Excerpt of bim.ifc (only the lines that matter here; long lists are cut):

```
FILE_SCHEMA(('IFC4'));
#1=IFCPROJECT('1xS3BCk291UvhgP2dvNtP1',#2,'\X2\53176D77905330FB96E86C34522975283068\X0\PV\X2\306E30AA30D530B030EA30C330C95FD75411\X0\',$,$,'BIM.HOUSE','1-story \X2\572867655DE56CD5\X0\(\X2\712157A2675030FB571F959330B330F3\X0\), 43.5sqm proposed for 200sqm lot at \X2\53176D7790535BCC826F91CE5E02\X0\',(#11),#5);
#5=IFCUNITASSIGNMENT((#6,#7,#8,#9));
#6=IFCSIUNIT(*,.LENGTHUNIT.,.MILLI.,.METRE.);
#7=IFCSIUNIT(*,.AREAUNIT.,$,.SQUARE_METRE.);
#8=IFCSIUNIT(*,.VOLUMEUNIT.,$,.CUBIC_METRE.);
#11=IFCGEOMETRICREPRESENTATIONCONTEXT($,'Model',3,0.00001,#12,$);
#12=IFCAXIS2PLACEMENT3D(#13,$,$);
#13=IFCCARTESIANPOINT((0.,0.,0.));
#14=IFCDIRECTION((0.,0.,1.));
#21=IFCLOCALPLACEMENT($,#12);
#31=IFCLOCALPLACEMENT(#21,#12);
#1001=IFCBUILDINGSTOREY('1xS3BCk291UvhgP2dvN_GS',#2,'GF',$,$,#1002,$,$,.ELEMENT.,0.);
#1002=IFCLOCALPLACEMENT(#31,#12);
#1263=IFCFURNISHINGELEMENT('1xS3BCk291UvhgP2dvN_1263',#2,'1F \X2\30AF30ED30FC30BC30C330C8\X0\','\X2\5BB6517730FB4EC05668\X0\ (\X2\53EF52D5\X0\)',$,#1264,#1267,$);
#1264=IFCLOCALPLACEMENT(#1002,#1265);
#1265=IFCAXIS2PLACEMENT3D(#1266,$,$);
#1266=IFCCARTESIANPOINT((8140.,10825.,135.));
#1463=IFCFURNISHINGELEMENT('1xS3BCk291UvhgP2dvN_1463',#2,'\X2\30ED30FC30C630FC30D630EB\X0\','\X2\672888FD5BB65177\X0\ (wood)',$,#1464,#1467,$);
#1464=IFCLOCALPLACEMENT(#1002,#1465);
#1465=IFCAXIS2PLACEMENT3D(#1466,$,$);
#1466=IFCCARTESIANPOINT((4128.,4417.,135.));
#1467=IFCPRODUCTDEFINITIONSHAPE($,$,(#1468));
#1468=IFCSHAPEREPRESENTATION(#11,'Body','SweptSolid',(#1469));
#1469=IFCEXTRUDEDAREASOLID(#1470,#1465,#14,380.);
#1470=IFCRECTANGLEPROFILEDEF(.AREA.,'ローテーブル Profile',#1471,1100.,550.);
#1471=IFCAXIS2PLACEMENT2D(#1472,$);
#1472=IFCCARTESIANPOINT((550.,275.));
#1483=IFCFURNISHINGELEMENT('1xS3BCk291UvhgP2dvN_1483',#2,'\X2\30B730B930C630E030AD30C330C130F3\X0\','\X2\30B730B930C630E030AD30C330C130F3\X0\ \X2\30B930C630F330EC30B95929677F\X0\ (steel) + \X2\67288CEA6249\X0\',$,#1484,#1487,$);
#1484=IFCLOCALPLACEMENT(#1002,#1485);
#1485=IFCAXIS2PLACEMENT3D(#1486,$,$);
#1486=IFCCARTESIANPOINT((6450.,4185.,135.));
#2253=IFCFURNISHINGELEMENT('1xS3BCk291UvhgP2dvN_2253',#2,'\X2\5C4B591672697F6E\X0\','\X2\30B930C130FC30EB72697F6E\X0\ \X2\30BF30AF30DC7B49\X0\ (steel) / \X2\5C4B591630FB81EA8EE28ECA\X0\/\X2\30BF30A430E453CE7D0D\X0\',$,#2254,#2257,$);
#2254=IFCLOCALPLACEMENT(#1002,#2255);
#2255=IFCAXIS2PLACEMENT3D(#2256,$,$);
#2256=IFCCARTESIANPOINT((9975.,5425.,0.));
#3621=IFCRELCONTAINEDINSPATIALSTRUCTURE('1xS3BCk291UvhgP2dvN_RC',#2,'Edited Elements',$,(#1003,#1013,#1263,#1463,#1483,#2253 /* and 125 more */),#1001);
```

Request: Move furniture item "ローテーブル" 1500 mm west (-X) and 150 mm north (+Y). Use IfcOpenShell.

```python
import ifcopenshell
import ifcopenshell.api.geometry
import ifcopenshell.util.placement
import ifcopenshell.util.unit

model = ifcopenshell.open("bim.ifc")
unit_scale = ifcopenshell.util.unit.calculate_unit_scale(model)

item = model.by_id(1463)
matrix = ifcopenshell.util.placement.get_local_placement(item.ObjectPlacement)
matrix[0, 3] -= 1.5 / unit_scale
matrix[1, 3] += 0.15 / unit_scale
ifcopenshell.api.geometry.edit_object_placement(model, product=item, matrix=matrix, is_si=False)

print(ifcopenshell.util.placement.get_local_placement(item.ObjectPlacement).round(3) + 0.0)

model.write("bim_edited.ifc")
```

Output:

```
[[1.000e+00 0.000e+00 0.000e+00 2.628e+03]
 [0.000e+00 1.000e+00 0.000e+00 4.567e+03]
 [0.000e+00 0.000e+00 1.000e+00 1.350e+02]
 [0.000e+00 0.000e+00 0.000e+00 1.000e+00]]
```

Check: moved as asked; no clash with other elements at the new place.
